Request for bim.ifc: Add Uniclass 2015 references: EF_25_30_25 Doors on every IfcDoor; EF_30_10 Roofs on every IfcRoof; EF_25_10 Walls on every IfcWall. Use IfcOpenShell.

First a look at what the model holds.

```python
import ifcopenshell

model = ifcopenshell.open("bim.ifc")
print(model.schema)
print("classifications:", [c.Name for c in model.by_type("IfcClassification")])
for ifc_class in ("IfcDoor", "IfcRoof", "IfcStair", "IfcWall", "IfcWindow"):
    print(ifc_class, len(model.by_type(ifc_class)))
```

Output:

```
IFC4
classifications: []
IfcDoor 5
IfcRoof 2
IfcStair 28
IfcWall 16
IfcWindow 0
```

```python
import ifcopenshell
import ifcopenshell.api.classification

model = ifcopenshell.open("bim.ifc")

system = ifcopenshell.api.classification.add_classification(model, classification="Uniclass 2015")

codes = {
    "IfcDoor": ("EF_25_30_25", "Doors"),
    "IfcRoof": ("EF_30_10", "Roofs"),
    "IfcWall": ("EF_25_10", "Walls"),
}
for ifc_class, (code, name) in codes.items():
    products = model.by_type(ifc_class)
    ifcopenshell.api.classification.add_reference(
        model, products=products, classification=system, identification=code, name=name
    )
    print(code, len(products))

model.write("bim_rev.ifc")
```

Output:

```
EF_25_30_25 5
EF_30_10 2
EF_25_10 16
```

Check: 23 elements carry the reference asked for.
